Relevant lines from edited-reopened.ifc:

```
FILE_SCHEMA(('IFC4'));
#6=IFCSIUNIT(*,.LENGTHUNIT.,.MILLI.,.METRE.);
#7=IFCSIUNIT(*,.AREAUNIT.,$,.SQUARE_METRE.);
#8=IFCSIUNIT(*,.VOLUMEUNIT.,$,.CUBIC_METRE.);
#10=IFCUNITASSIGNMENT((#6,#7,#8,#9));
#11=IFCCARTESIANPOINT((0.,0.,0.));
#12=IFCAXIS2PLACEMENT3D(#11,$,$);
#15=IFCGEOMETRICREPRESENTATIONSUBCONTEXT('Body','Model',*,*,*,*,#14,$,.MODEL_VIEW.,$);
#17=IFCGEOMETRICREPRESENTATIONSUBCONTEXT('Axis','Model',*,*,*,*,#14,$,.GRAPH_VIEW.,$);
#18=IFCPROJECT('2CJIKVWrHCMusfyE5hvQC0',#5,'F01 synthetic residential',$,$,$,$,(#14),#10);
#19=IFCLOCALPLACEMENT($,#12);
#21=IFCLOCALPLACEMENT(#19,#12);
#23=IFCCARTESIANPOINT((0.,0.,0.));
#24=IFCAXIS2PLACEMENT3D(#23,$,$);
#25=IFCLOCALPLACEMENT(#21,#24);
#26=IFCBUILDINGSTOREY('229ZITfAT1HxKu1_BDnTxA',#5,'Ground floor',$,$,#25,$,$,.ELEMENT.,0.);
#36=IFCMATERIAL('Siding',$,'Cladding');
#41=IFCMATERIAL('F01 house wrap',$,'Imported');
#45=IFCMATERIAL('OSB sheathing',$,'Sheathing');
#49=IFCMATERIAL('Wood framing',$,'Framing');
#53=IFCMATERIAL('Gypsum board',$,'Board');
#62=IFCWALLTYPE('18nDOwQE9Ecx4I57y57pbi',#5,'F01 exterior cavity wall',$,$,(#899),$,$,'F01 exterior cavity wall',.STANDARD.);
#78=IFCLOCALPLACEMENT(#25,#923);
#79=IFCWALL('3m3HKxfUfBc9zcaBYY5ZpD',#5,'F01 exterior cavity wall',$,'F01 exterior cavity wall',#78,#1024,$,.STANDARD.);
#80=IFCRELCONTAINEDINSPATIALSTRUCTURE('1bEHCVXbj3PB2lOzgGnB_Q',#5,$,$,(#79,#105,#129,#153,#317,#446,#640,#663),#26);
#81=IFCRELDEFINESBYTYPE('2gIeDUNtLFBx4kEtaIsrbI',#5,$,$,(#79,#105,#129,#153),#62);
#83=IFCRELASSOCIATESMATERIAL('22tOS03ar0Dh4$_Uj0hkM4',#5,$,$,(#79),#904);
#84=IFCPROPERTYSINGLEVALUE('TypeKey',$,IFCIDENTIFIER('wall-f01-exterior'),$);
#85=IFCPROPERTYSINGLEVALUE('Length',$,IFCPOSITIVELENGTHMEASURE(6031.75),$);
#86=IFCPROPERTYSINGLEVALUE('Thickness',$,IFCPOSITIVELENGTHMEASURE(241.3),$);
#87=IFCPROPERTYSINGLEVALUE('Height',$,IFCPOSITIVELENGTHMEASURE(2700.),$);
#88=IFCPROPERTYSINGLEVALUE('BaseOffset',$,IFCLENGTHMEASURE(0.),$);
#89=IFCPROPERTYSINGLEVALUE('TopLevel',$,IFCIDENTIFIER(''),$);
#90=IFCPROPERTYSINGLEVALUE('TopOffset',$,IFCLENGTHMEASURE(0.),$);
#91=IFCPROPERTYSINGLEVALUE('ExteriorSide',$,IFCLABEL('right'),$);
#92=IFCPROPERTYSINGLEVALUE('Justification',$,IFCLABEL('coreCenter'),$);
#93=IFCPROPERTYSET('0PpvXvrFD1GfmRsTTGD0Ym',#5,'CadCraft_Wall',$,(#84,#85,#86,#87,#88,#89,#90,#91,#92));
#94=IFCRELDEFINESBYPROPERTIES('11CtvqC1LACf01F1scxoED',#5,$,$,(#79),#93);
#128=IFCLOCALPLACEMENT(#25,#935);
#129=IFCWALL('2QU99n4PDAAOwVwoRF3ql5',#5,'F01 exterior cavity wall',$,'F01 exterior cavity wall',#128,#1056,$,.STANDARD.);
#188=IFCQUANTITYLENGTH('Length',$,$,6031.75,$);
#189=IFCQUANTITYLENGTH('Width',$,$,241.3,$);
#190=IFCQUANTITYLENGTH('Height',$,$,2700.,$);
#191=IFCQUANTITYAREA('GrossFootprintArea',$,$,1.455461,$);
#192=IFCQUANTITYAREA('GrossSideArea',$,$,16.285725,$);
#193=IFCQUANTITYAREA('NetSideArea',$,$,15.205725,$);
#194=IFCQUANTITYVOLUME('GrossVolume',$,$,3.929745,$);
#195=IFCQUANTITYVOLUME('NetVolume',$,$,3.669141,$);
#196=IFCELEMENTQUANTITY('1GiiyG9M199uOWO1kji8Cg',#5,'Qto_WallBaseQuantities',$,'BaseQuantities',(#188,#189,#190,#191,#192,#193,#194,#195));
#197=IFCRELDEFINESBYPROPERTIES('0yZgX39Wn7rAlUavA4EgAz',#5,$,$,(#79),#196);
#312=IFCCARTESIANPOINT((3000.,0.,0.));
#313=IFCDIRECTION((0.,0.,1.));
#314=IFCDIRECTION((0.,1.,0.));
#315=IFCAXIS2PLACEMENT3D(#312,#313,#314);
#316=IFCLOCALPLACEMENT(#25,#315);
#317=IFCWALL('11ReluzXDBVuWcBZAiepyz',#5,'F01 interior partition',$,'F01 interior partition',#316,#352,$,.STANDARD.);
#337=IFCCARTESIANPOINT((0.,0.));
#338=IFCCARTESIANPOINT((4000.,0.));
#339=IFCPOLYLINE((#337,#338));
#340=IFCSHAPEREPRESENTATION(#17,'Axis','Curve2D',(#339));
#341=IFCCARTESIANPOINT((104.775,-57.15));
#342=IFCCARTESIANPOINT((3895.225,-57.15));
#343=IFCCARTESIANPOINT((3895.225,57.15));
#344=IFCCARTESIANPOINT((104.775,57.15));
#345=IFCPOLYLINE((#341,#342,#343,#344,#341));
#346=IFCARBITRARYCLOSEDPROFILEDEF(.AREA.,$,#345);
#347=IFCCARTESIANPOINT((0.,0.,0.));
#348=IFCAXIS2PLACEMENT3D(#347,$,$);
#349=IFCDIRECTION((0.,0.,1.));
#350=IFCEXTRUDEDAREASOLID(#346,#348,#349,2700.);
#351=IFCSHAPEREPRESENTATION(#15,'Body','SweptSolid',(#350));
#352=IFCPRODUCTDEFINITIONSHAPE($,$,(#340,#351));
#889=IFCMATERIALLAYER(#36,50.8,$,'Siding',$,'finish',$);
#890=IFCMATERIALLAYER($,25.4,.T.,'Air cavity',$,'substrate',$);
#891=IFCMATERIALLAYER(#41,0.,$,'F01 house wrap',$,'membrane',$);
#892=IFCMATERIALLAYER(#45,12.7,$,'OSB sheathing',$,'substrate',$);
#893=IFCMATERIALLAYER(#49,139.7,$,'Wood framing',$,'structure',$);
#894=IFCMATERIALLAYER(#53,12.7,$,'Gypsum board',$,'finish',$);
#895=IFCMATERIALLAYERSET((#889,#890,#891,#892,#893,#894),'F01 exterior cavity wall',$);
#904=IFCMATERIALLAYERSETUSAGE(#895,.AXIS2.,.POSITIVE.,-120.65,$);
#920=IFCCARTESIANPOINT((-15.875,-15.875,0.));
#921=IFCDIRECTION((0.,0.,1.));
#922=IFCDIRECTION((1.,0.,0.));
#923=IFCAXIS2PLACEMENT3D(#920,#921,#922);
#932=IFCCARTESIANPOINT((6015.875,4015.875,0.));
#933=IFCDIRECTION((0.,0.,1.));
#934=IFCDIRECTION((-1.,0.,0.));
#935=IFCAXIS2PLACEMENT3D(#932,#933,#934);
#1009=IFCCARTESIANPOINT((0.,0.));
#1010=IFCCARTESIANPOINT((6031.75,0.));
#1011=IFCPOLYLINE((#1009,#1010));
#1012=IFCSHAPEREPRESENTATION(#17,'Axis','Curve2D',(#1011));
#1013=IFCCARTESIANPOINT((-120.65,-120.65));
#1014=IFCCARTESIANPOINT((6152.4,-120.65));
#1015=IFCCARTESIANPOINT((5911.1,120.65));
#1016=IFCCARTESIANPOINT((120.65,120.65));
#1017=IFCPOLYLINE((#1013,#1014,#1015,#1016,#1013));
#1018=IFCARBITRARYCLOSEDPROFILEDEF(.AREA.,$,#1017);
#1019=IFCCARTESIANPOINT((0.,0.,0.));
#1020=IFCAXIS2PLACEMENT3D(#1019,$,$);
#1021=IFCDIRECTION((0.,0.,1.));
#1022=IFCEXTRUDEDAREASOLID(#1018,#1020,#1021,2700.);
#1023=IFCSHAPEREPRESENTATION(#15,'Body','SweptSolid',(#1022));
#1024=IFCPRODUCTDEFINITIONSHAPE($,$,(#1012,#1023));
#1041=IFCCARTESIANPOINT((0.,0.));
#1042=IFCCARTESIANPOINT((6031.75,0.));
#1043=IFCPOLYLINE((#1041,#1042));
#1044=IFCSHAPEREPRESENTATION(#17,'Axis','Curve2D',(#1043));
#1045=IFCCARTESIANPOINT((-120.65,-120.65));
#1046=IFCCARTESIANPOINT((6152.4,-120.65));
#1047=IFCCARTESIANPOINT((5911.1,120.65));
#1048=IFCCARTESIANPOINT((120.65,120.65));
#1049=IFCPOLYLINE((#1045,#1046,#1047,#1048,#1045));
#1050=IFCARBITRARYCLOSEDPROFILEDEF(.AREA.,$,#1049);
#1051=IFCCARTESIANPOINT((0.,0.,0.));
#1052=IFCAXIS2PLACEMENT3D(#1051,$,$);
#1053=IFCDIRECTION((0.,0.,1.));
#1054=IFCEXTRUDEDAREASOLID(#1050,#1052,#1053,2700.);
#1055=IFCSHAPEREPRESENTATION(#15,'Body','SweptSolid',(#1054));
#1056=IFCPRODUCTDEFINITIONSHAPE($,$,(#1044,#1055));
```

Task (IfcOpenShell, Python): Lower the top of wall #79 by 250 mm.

```python
import ifcopenshell
import ifcopenshell.api.pset
import ifcopenshell.geom
import ifcopenshell.util.element
import ifcopenshell.util.representation
import ifcopenshell.util.shape
import ifcopenshell.util.unit

model = ifcopenshell.open("edited-reopened.ifc")
unit_scale = ifcopenshell.util.unit.calculate_unit_scale(model)
area_scale = ifcopenshell.util.unit.calculate_unit_scale(model, "AREAUNIT")
volume_scale = ifcopenshell.util.unit.calculate_unit_scale(model, "VOLUMEUNIT")
settings = ifcopenshell.geom.settings()


def volume(element):
    """Net volume in cubic metres, openings subtracted."""
    shape = ifcopenshell.geom.create_shape(settings, element)
    return ifcopenshell.util.shape.get_volume(shape.geometry)


wall = model.by_id(79)
before = volume(wall)

body = ifcopenshell.util.representation.get_representation(wall, "Model", "Body")
solid = body.Items[0]
old_height = solid.Depth
solid.Depth -= 0.25 / unit_scale
after = volume(wall)
thickness = 0.2413  # wall thickness in metres

# Update the stored height, areas and volumes.
pset = model.by_id(ifcopenshell.util.element.get_pset(wall, "CadCraft_Wall", should_inherit=False)["id"])
ifcopenshell.api.pset.edit_pset(model, pset=pset, properties={
    "Height": model.create_entity("IfcPositiveLengthMeasure", solid.Depth),
})
qto = model.by_id(ifcopenshell.util.element.get_pset(wall, "Qto_WallBaseQuantities", should_inherit=False)["id"])
ifcopenshell.api.pset.edit_qto(model, qto=qto, properties={
    "Height": solid.Depth,
    "GrossSideArea": ifcopenshell.util.element.get_pset(wall, "Qto_WallBaseQuantities", "GrossSideArea") * solid.Depth / old_height,
    "NetSideArea": after / thickness / area_scale,
    "GrossVolume": ifcopenshell.util.element.get_pset(wall, "Qto_WallBaseQuantities", "GrossVolume") * solid.Depth / old_height,
    "NetVolume": after / volume_scale,
})

print(f"height {old_height:g} -> {solid.Depth:g}, volume {before:.3f} -> {after:.3f} m3")

model.write("edited-reopened-out.ifc")
```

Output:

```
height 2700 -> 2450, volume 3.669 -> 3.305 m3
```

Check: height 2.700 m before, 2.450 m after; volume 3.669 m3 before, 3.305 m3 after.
